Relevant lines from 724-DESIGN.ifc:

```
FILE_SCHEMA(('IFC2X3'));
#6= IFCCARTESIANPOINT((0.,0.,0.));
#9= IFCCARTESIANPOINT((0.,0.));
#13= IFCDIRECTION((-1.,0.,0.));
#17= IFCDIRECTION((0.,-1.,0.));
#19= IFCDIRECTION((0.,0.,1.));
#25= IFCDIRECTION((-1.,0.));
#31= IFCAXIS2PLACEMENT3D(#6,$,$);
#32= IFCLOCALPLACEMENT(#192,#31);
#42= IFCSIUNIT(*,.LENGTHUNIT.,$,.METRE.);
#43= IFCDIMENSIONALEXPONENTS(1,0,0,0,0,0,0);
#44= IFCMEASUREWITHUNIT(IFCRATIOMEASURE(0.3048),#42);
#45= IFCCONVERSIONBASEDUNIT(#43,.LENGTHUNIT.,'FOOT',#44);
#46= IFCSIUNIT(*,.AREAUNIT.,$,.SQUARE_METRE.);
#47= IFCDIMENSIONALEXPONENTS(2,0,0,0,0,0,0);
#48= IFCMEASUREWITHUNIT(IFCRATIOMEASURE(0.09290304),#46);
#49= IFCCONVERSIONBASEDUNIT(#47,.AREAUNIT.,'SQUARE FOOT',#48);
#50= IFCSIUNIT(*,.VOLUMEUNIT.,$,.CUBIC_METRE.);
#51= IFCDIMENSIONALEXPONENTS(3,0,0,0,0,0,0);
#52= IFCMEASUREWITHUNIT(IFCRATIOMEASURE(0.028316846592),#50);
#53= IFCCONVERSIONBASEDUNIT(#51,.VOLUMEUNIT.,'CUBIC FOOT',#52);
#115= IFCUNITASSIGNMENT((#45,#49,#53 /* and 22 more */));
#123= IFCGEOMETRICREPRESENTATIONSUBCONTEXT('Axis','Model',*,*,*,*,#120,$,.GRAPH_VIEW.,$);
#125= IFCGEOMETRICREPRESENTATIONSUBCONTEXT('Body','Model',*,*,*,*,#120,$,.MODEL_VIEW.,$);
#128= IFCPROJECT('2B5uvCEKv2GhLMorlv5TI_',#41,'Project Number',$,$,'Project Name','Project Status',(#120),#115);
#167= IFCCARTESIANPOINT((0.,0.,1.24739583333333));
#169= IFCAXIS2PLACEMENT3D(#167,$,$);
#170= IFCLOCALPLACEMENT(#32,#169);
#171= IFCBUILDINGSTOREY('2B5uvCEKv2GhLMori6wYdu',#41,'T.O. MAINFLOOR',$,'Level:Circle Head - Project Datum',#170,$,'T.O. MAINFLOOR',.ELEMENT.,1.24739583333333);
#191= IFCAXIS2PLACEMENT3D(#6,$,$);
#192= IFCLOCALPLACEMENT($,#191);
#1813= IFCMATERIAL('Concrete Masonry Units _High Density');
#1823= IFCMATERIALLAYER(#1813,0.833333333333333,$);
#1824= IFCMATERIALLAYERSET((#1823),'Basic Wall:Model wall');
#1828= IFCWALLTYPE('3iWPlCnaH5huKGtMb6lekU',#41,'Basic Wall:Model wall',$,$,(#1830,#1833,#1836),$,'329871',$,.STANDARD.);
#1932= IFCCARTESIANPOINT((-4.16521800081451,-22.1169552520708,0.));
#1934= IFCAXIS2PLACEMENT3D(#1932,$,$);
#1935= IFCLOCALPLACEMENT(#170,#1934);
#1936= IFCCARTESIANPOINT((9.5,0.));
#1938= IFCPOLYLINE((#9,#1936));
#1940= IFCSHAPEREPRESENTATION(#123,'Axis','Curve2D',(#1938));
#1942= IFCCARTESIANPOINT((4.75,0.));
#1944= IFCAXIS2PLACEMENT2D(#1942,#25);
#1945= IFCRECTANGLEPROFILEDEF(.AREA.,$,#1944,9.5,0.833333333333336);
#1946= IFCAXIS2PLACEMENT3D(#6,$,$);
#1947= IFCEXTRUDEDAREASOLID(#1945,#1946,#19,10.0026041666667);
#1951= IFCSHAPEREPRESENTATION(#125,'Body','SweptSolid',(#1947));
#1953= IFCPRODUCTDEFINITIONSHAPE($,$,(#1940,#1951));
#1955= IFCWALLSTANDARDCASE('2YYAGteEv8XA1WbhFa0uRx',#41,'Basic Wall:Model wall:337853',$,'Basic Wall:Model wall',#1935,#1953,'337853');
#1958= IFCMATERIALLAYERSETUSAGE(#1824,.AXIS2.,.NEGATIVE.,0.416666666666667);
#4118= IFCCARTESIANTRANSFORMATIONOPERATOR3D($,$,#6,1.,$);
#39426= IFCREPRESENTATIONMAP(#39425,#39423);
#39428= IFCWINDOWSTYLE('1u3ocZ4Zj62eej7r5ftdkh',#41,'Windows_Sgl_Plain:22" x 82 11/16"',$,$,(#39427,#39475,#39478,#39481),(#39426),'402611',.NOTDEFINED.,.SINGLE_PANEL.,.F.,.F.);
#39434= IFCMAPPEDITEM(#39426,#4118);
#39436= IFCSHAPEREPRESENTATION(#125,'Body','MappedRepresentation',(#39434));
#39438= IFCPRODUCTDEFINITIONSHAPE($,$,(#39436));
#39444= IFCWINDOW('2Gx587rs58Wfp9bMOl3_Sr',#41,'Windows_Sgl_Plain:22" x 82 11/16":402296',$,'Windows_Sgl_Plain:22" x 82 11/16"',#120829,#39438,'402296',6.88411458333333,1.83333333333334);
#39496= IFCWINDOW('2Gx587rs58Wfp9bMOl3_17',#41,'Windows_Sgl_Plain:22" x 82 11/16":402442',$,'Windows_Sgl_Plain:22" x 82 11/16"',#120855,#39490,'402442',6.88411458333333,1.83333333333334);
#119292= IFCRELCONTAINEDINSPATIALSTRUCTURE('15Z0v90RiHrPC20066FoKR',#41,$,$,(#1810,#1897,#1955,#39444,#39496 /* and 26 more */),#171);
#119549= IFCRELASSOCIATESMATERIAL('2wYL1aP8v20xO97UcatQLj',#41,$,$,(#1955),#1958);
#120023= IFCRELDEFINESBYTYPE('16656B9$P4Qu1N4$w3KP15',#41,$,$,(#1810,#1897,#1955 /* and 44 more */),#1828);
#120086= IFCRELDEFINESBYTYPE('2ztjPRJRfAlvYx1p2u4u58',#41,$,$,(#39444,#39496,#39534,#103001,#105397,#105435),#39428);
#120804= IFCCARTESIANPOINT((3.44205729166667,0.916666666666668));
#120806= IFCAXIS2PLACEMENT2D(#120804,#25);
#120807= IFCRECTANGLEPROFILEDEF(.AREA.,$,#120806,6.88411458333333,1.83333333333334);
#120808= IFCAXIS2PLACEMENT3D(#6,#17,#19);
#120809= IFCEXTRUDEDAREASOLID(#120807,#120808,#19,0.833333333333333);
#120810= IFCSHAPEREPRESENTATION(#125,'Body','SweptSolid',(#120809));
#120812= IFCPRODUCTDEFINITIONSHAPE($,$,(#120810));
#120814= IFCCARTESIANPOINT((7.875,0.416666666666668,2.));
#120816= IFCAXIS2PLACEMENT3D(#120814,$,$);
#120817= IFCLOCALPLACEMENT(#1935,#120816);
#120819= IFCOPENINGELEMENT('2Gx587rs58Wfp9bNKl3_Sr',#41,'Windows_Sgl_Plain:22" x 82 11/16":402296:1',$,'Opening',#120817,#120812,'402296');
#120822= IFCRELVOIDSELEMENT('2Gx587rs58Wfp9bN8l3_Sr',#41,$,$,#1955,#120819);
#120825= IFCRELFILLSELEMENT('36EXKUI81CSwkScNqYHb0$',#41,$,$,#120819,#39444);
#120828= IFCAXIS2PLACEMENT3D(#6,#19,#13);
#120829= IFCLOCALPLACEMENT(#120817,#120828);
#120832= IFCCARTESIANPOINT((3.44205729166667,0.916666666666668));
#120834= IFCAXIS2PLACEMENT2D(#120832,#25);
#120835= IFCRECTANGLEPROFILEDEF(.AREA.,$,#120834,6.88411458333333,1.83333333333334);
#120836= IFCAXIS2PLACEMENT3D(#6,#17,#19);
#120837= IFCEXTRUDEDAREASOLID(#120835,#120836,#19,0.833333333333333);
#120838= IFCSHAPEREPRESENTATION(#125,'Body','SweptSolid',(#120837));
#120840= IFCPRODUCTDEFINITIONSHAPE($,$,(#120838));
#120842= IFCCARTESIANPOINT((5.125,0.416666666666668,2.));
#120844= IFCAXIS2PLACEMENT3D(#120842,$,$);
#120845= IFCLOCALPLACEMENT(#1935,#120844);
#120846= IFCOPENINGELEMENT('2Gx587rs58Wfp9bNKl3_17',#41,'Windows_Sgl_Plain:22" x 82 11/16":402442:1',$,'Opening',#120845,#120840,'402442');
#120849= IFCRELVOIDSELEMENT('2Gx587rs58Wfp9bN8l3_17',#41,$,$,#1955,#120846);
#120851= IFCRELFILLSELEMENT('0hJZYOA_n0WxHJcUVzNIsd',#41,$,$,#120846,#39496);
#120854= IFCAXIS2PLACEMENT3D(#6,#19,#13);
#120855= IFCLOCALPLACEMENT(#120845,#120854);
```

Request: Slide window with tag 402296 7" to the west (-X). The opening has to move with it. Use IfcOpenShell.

```python
import ifcopenshell
import ifcopenshell.api.geometry
import ifcopenshell.util.placement
import ifcopenshell.util.unit

model = ifcopenshell.open("724-DESIGN.ifc")
unit_scale = ifcopenshell.util.unit.calculate_unit_scale(model)

window = model.by_id(39444)
opening = window.FillsVoids[0].RelatingOpeningElement
wall = opening.VoidsElements[0].RelatingBuildingElement

wall_matrix = ifcopenshell.util.placement.get_local_placement(wall.ObjectPlacement)
shift = wall_matrix[:3, 0] * -7 * 0.0254 / unit_scale
before = ifcopenshell.util.placement.get_local_placement(window.ObjectPlacement)[:3, 3].copy()

# The window is placed relative to its opening, so it follows when the opening moves.
matrix = ifcopenshell.util.placement.get_local_placement(opening.ObjectPlacement)
matrix[:3, 3] += shift
ifcopenshell.api.geometry.edit_object_placement(
    model, product=opening, matrix=matrix, is_si=False, should_transform_children=True
)

after = ifcopenshell.util.placement.get_local_placement(window.ObjectPlacement)[:3, 3]
print("window moved by", (after - before).round(3) + 0.0)

model.write("724-DESIGN_v2.ifc")
```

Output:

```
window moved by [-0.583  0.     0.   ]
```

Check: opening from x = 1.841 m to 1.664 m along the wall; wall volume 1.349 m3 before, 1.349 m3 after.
